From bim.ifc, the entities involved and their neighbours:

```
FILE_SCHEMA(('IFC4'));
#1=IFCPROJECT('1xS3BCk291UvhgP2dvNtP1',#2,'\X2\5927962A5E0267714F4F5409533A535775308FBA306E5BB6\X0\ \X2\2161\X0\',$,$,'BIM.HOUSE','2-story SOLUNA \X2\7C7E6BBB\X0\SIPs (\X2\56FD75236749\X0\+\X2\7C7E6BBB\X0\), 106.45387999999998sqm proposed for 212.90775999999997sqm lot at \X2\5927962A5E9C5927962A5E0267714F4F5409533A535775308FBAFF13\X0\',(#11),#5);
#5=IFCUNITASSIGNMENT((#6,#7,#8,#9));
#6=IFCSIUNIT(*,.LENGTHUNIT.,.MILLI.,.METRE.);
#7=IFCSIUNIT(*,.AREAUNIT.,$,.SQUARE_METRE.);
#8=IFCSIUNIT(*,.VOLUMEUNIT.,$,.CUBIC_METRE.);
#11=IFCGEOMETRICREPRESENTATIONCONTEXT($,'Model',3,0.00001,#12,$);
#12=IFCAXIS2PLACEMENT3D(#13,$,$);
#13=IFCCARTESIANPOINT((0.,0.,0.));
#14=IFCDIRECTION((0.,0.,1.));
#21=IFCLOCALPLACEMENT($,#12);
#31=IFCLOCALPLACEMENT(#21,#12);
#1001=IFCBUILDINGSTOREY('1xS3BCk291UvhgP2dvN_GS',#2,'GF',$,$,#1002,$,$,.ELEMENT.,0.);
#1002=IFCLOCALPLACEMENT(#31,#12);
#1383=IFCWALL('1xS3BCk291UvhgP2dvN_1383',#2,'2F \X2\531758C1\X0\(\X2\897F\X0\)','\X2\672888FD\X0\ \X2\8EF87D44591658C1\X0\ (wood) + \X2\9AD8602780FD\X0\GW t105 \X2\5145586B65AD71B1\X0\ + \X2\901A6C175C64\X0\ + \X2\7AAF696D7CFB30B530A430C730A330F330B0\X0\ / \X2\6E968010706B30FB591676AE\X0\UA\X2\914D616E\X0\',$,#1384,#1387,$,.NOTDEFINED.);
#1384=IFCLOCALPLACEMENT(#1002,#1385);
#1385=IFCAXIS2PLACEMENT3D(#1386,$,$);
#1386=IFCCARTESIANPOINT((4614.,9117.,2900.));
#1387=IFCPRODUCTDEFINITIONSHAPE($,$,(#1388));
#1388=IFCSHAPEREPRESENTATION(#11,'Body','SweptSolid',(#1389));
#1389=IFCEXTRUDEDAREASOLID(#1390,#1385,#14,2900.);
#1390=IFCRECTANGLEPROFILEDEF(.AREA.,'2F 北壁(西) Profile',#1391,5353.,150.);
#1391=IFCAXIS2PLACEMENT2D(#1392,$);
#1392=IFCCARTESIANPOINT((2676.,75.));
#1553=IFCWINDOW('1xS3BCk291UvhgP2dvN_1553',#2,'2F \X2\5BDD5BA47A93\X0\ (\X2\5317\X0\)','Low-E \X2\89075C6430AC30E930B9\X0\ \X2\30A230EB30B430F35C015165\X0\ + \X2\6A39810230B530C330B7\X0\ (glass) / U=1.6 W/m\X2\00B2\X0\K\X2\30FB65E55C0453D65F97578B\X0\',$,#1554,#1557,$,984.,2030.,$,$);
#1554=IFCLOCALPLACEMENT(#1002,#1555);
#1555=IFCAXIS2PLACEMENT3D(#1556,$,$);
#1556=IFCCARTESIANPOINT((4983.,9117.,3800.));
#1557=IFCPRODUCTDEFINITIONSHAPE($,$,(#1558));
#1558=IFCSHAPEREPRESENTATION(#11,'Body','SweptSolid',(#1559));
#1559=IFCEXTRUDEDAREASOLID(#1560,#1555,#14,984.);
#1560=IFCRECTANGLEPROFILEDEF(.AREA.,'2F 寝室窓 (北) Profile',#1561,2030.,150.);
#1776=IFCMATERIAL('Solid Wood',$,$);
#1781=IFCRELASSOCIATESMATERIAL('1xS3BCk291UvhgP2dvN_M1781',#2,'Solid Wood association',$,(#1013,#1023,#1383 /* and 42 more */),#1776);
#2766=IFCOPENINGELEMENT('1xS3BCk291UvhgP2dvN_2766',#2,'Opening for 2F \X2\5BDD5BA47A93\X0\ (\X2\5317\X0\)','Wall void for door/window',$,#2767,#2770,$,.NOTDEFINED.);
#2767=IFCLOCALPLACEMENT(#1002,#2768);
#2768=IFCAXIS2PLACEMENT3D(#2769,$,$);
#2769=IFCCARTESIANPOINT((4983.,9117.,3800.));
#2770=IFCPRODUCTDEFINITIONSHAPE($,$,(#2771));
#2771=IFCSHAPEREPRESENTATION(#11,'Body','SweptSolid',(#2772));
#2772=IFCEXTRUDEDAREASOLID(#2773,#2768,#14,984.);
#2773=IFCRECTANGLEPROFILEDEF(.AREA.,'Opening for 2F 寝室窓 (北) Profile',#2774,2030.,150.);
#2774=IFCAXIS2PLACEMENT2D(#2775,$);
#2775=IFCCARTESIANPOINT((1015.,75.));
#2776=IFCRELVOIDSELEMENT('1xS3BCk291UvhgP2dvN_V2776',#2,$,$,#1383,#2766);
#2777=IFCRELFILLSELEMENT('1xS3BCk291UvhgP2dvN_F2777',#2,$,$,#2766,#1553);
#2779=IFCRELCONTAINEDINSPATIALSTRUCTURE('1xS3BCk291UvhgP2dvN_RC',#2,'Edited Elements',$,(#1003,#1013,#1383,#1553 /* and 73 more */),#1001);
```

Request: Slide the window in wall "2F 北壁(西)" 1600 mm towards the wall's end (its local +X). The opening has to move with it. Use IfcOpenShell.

```python
import ifcopenshell
import ifcopenshell.api.geometry
import ifcopenshell.util.placement

model = ifcopenshell.open("bim.ifc")

window = model.by_id(1553)
opening = window.FillsVoids[0].RelatingOpeningElement
wall = opening.VoidsElements[0].RelatingBuildingElement

wall_matrix = ifcopenshell.util.placement.get_local_placement(wall.ObjectPlacement)
shift = wall_matrix[:3, 0] * 1600.0
before = ifcopenshell.util.placement.get_local_placement(window.ObjectPlacement)[:3, 3].copy()

# The window is not placed relative to its opening, so move both.
for product in (opening, window):
    matrix = ifcopenshell.util.placement.get_local_placement(product.ObjectPlacement)
    matrix[:3, 3] += shift
    ifcopenshell.api.geometry.edit_object_placement(model, product=product, matrix=matrix, is_si=False)

after = ifcopenshell.util.placement.get_local_placement(window.ObjectPlacement)[:3, 3]
print("window moved by", (after - before).round(3) + 0.0)

model.write("bim_v2.ifc")
```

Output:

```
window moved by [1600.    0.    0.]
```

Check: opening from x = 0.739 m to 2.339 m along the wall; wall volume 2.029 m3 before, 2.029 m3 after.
